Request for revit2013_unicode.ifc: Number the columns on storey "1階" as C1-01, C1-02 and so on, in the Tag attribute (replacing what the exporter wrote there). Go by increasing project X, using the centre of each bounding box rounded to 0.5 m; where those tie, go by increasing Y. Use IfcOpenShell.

First a look at what the model holds.

```python
import ifcopenshell
import ifcopenshell.util.element
import ifcopenshell.util.placement

model = ifcopenshell.open("revit2013_unicode.ifc")
print(model.schema)
storey = next(s for s in model.by_type("IfcBuildingStorey") if s.Name == "1階")
columns = [e for e in ifcopenshell.util.element.get_decomposition(storey) if e.is_a("IfcColumn")]
for e in sorted(columns, key=lambda e: e.id()):
    origin = ifcopenshell.util.placement.get_local_placement(e.ObjectPlacement)[:3, 3]
    print(e.id(), e.Tag, e.Name, origin.round(2) + 0.0, sep=" | ")
```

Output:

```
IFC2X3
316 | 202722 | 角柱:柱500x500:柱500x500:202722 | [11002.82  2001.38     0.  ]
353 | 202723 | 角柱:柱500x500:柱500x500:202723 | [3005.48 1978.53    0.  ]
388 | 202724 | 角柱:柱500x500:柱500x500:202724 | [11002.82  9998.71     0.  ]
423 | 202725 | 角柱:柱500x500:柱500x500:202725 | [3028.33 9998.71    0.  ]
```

```python
import ifcopenshell
import ifcopenshell.geom
import ifcopenshell.util.element
import ifcopenshell.util.shape

model = ifcopenshell.open("revit2013_unicode.ifc")
settings = ifcopenshell.geom.settings()
settings.set("use-world-coords", True)


def centre(element):
    shape = ifcopenshell.geom.create_shape(settings, element)
    return ifcopenshell.util.shape.get_bbox_centroid(shape.geometry)


storey = next(s for s in model.by_type("IfcBuildingStorey") if s.Name == "1階")
columns = [e for e in ifcopenshell.util.element.get_decomposition(storey) if e.is_a("IfcColumn")]

# Insertion points can sit at a corner or the storey origin, so sort by the geometry (in metres).
centres = {e: centre(e) for e in columns}
columns.sort(key=lambda e: (round(centres[e][0] / 0.5), centres[e][1]))

for i, e in enumerate(columns, start=1):
    number = f"C1-{i:02d}"
    e.Tag = number
    print(e.id(), number)

model.write("revit2013_unicode_edited.ifc")
```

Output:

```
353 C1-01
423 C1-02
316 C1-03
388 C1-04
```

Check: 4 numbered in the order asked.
